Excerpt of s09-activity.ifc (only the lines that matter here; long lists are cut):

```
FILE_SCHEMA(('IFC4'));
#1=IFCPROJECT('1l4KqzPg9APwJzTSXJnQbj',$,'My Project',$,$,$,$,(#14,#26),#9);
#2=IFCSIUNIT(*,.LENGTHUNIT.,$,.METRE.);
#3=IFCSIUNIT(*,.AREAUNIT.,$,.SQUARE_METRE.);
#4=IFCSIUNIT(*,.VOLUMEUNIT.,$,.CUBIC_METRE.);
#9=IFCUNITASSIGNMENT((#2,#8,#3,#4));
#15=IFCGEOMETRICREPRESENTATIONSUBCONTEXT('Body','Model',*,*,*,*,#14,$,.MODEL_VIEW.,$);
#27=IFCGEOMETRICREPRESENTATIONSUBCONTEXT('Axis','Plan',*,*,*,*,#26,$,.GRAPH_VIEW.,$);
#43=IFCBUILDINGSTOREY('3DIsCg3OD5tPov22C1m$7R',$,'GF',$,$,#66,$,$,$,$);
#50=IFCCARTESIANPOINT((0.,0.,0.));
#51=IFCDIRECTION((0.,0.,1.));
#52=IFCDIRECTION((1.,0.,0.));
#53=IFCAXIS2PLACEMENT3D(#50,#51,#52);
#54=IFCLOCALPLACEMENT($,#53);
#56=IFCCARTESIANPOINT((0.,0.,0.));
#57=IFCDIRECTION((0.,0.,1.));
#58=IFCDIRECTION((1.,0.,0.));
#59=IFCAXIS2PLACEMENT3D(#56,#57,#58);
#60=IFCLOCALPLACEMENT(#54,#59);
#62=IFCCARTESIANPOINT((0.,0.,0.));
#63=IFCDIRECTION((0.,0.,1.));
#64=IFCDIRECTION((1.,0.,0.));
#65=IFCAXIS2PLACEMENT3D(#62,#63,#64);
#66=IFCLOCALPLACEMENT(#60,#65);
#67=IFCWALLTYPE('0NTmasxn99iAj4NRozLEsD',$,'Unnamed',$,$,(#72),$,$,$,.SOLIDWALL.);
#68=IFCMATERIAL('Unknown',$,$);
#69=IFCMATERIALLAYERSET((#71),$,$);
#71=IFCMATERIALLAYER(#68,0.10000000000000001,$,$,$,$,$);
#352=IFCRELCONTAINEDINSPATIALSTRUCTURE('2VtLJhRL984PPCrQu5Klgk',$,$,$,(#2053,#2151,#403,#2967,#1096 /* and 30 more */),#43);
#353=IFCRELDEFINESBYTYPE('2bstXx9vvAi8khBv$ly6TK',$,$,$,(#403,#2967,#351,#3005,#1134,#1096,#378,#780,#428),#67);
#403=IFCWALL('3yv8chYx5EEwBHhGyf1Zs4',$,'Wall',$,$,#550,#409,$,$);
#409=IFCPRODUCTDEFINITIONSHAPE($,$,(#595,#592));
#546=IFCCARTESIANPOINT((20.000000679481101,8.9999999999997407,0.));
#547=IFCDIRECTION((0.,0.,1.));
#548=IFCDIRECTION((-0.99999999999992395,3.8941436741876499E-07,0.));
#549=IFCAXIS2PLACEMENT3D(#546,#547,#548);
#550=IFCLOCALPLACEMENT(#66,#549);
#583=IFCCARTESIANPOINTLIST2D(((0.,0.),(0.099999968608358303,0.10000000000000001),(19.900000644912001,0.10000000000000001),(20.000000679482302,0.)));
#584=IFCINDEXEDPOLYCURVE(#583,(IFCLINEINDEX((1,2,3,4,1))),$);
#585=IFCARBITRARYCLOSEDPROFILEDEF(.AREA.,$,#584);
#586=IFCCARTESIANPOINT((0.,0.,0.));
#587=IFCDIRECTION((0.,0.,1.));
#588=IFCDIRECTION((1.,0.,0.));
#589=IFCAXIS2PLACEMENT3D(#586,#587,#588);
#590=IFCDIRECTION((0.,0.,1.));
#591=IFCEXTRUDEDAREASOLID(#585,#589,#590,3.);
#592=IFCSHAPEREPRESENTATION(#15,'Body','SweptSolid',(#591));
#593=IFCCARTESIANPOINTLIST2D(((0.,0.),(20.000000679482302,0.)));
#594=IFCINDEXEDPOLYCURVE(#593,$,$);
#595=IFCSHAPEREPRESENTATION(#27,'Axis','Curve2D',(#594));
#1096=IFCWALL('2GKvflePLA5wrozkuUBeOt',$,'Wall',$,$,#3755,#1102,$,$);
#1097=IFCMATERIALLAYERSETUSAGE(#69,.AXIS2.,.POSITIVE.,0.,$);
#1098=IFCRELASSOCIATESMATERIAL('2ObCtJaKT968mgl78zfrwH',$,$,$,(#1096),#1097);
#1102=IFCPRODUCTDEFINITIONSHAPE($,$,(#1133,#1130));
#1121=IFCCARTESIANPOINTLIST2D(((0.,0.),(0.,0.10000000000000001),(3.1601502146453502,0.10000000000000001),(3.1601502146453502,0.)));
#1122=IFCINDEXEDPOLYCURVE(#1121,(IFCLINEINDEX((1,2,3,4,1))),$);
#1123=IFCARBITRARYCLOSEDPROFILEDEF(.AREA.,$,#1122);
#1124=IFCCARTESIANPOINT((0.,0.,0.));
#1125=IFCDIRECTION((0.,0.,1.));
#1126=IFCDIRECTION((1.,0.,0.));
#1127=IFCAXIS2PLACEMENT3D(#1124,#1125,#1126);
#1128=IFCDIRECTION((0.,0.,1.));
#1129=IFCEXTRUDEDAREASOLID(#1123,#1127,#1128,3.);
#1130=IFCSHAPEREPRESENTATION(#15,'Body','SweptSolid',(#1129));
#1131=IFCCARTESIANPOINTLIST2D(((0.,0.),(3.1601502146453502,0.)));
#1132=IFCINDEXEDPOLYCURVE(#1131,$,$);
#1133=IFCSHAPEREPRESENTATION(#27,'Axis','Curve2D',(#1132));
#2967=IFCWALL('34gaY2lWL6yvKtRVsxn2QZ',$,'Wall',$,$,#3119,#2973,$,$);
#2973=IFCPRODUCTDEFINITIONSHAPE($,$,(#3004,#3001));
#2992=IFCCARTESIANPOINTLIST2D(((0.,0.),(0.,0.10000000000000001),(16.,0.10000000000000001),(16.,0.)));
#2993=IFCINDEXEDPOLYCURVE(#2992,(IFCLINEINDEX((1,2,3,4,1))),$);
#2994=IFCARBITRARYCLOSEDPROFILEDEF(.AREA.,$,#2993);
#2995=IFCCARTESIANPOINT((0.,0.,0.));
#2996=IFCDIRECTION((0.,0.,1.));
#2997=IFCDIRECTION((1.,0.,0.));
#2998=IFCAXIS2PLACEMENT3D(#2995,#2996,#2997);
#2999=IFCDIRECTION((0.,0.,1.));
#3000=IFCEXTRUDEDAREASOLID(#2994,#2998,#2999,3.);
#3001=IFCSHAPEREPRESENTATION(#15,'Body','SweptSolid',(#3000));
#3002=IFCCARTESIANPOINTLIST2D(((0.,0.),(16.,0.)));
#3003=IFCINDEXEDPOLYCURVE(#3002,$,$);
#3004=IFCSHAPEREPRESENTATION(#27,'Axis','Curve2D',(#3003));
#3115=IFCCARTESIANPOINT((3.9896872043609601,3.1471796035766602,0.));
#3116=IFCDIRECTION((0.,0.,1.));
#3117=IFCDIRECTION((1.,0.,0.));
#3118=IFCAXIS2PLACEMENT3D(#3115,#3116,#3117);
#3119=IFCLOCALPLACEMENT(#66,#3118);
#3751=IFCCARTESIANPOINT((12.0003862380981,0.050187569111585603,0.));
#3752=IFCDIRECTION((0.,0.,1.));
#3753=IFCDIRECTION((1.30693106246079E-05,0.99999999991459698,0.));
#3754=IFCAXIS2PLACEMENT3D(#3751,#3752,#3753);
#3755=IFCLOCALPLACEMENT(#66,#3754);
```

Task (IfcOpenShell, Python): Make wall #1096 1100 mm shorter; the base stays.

```python
import ifcopenshell
import ifcopenshell.geom
import ifcopenshell.util.representation
import ifcopenshell.util.shape
import ifcopenshell.util.unit

model = ifcopenshell.open("s09-activity.ifc")
unit_scale = ifcopenshell.util.unit.calculate_unit_scale(model)
settings = ifcopenshell.geom.settings()


def volume(element):
    """Net volume in cubic metres, openings subtracted."""
    shape = ifcopenshell.geom.create_shape(settings, element)
    return ifcopenshell.util.shape.get_volume(shape.geometry)


wall = model.by_guid("2GKvflePLA5wrozkuUBeOt")
before = volume(wall)

body = ifcopenshell.util.representation.get_representation(wall, "Model", "Body")
solid = body.Items[0]
old_height = solid.Depth
solid.Depth -= 1.1 / unit_scale
after = volume(wall)

print(f"height {old_height:g} -> {solid.Depth:g}, volume {before:.3f} -> {after:.3f} m3")

model.write("s09-activity-out.ifc")
```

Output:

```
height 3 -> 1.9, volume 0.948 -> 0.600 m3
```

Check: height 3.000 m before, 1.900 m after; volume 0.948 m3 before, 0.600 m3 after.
